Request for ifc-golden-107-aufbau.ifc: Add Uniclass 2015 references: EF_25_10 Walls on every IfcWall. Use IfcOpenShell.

First a look at what the model holds.

```python
import ifcopenshell

model = ifcopenshell.open("ifc-golden-107-aufbau.ifc")
print(model.schema)
print("classifications:", [c.Name for c in model.by_type("IfcClassification")])
for ifc_class in ("IfcDoor", "IfcRoof", "IfcStair", "IfcWall", "IfcWindow"):
    print(ifc_class, len(model.by_type(ifc_class)))
```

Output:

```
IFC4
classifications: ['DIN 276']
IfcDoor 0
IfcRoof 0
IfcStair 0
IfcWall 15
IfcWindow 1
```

```python
import ifcopenshell
import ifcopenshell.api.classification

model = ifcopenshell.open("ifc-golden-107-aufbau.ifc")

system = ifcopenshell.api.classification.add_classification(model, classification="Uniclass 2015")

codes = {
    "IfcWall": ("EF_25_10", "Walls"),
}
for ifc_class, (code, name) in codes.items():
    products = model.by_type(ifc_class)
    ifcopenshell.api.classification.add_reference(
        model, products=products, classification=system, identification=code, name=name
    )
    print(code, len(products))

model.write("ifc-golden-107-aufbau_rev.ifc")
```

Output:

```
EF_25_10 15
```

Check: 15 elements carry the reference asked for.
